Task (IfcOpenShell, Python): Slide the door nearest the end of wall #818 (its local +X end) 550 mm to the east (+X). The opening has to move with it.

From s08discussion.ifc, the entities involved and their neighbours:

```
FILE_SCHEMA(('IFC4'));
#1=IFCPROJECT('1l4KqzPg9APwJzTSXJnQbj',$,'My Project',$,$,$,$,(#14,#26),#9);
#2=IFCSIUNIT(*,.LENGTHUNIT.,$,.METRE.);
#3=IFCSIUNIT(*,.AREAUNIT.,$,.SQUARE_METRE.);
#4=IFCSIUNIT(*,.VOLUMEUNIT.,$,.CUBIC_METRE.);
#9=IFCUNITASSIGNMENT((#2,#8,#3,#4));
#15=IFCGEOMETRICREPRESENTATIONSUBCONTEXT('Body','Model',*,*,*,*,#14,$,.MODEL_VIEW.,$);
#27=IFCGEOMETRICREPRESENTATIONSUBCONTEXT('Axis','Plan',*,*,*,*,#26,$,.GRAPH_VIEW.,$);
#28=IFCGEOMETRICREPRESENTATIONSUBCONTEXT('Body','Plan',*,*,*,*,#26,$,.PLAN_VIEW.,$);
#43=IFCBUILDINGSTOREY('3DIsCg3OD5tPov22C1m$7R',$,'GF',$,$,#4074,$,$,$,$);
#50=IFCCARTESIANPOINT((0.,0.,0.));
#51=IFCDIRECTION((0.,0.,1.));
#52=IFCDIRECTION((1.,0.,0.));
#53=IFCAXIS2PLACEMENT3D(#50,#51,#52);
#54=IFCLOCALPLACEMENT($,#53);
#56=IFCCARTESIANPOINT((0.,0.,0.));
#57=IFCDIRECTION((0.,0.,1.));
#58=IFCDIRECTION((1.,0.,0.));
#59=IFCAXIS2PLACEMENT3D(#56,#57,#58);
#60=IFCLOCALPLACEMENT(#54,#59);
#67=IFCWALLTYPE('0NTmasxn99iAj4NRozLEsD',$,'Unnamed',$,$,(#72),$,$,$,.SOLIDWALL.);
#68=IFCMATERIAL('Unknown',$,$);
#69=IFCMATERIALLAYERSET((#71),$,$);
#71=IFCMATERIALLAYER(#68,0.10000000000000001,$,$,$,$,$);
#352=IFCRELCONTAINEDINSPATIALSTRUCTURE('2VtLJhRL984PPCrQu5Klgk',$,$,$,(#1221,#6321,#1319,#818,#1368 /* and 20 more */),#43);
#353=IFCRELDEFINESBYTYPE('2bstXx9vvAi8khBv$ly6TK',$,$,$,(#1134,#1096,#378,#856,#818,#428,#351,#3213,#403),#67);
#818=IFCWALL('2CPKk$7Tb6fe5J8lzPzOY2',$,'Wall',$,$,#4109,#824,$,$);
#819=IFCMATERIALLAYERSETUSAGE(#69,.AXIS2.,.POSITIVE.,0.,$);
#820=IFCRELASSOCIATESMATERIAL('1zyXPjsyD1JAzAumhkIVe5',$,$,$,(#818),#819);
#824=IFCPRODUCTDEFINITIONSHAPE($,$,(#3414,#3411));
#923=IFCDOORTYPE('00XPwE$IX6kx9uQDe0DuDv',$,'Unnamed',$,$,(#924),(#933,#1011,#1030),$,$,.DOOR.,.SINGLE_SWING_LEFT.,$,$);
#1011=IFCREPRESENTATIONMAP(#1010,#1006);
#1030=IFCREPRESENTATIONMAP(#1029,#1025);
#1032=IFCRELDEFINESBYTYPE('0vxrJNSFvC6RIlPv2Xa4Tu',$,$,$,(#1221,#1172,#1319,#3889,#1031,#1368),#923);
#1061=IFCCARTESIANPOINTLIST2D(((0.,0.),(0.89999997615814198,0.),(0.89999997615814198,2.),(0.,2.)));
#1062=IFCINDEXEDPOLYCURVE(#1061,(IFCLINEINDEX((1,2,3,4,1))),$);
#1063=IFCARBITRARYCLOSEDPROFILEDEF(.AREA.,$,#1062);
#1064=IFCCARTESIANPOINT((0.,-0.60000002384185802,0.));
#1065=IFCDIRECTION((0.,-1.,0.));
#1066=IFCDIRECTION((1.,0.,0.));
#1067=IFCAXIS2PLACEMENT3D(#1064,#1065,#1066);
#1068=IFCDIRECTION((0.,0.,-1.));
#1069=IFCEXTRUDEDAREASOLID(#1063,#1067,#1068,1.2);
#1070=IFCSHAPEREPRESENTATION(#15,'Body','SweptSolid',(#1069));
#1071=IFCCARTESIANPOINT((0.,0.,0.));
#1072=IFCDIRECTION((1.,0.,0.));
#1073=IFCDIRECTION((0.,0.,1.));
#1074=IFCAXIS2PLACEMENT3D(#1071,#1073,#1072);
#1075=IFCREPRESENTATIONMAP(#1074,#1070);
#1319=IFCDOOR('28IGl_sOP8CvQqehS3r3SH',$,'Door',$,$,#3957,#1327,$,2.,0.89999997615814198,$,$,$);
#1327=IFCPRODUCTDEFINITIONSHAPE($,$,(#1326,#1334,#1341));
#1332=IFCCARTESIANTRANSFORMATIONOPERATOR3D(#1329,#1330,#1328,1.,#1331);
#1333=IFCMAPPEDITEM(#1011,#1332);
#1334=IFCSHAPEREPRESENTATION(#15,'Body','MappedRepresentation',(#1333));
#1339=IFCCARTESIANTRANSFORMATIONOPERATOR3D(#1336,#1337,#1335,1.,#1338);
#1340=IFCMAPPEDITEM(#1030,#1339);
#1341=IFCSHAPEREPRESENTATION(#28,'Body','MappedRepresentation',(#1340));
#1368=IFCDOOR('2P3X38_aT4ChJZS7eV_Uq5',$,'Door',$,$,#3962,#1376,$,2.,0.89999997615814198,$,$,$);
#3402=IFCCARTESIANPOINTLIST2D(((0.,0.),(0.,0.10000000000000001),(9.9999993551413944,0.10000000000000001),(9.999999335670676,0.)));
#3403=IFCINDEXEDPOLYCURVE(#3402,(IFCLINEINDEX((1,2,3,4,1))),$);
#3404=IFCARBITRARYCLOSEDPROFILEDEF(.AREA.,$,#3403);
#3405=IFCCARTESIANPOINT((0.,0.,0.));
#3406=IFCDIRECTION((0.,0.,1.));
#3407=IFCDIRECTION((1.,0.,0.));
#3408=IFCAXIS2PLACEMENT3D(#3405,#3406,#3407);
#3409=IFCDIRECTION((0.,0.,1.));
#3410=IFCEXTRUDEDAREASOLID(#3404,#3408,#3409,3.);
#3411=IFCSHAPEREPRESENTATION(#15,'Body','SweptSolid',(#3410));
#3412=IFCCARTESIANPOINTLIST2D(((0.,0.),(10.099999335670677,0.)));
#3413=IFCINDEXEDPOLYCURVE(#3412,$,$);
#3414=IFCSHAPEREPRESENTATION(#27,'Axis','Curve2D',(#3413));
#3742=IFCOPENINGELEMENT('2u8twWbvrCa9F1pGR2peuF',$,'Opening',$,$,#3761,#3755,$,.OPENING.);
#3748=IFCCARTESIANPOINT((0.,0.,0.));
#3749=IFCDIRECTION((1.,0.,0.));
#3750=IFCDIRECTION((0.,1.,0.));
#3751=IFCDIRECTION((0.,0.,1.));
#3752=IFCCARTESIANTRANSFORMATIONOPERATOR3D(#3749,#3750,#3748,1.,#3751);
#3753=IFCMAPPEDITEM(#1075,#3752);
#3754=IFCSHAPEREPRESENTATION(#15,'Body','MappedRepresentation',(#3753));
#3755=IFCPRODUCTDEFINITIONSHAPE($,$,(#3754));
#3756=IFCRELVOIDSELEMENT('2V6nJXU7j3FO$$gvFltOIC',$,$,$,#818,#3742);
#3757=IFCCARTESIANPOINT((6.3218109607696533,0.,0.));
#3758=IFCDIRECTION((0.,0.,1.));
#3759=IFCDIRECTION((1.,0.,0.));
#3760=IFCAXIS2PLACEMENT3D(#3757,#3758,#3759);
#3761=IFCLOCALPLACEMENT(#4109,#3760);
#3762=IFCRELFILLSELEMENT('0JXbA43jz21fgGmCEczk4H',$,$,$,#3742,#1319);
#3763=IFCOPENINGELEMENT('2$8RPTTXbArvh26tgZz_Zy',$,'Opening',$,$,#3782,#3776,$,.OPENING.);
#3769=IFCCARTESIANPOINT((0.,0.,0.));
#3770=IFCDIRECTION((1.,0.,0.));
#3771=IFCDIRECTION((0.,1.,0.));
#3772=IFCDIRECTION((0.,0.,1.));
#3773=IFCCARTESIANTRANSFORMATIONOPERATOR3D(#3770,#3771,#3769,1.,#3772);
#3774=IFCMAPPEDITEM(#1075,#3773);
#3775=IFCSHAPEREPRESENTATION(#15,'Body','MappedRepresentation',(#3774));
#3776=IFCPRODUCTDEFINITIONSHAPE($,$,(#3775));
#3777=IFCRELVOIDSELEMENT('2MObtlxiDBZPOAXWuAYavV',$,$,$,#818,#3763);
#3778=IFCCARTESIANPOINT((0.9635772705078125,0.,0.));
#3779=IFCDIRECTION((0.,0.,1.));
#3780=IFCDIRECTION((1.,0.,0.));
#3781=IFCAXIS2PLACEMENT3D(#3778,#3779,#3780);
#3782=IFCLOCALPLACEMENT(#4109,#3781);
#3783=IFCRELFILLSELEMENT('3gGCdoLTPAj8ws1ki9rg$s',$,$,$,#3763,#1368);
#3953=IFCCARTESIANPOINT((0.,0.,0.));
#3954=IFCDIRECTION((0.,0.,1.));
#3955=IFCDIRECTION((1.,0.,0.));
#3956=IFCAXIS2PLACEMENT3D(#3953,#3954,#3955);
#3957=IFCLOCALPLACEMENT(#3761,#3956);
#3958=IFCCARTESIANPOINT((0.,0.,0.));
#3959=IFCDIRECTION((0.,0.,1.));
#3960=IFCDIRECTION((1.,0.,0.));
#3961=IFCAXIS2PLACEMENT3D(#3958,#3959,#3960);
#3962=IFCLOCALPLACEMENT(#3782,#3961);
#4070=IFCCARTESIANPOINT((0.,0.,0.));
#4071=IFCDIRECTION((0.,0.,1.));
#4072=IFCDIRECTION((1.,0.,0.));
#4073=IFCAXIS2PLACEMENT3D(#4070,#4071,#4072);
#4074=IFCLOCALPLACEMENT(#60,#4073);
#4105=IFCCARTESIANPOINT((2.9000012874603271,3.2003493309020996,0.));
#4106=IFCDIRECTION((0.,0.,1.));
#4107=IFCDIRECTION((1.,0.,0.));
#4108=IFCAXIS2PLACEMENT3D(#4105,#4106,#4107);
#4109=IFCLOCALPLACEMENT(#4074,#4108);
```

```python
import ifcopenshell
import ifcopenshell.api.geometry
import ifcopenshell.util.placement

model = ifcopenshell.open("s08discussion.ifc")

door = model.by_guid("28IGl_sOP8CvQqehS3r3SH")
opening = door.FillsVoids[0].RelatingOpeningElement
wall = opening.VoidsElements[0].RelatingBuildingElement

wall_matrix = ifcopenshell.util.placement.get_local_placement(wall.ObjectPlacement)
shift = wall_matrix[:3, 0] * 0.55
before = ifcopenshell.util.placement.get_local_placement(door.ObjectPlacement)[:3, 3].copy()

# The door is placed relative to its opening, so it follows when the opening moves.
matrix = ifcopenshell.util.placement.get_local_placement(opening.ObjectPlacement)
matrix[:3, 3] += shift
ifcopenshell.api.geometry.edit_object_placement(
    model, product=opening, matrix=matrix, is_si=False, should_transform_children=True
)

after = ifcopenshell.util.placement.get_local_placement(door.ObjectPlacement)[:3, 3]
print("door moved by", (after - before).round(3) + 0.0)

model.write("s08discussion-out.ifc")
```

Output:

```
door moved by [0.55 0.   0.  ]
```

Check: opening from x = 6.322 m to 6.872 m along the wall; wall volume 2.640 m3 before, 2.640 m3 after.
